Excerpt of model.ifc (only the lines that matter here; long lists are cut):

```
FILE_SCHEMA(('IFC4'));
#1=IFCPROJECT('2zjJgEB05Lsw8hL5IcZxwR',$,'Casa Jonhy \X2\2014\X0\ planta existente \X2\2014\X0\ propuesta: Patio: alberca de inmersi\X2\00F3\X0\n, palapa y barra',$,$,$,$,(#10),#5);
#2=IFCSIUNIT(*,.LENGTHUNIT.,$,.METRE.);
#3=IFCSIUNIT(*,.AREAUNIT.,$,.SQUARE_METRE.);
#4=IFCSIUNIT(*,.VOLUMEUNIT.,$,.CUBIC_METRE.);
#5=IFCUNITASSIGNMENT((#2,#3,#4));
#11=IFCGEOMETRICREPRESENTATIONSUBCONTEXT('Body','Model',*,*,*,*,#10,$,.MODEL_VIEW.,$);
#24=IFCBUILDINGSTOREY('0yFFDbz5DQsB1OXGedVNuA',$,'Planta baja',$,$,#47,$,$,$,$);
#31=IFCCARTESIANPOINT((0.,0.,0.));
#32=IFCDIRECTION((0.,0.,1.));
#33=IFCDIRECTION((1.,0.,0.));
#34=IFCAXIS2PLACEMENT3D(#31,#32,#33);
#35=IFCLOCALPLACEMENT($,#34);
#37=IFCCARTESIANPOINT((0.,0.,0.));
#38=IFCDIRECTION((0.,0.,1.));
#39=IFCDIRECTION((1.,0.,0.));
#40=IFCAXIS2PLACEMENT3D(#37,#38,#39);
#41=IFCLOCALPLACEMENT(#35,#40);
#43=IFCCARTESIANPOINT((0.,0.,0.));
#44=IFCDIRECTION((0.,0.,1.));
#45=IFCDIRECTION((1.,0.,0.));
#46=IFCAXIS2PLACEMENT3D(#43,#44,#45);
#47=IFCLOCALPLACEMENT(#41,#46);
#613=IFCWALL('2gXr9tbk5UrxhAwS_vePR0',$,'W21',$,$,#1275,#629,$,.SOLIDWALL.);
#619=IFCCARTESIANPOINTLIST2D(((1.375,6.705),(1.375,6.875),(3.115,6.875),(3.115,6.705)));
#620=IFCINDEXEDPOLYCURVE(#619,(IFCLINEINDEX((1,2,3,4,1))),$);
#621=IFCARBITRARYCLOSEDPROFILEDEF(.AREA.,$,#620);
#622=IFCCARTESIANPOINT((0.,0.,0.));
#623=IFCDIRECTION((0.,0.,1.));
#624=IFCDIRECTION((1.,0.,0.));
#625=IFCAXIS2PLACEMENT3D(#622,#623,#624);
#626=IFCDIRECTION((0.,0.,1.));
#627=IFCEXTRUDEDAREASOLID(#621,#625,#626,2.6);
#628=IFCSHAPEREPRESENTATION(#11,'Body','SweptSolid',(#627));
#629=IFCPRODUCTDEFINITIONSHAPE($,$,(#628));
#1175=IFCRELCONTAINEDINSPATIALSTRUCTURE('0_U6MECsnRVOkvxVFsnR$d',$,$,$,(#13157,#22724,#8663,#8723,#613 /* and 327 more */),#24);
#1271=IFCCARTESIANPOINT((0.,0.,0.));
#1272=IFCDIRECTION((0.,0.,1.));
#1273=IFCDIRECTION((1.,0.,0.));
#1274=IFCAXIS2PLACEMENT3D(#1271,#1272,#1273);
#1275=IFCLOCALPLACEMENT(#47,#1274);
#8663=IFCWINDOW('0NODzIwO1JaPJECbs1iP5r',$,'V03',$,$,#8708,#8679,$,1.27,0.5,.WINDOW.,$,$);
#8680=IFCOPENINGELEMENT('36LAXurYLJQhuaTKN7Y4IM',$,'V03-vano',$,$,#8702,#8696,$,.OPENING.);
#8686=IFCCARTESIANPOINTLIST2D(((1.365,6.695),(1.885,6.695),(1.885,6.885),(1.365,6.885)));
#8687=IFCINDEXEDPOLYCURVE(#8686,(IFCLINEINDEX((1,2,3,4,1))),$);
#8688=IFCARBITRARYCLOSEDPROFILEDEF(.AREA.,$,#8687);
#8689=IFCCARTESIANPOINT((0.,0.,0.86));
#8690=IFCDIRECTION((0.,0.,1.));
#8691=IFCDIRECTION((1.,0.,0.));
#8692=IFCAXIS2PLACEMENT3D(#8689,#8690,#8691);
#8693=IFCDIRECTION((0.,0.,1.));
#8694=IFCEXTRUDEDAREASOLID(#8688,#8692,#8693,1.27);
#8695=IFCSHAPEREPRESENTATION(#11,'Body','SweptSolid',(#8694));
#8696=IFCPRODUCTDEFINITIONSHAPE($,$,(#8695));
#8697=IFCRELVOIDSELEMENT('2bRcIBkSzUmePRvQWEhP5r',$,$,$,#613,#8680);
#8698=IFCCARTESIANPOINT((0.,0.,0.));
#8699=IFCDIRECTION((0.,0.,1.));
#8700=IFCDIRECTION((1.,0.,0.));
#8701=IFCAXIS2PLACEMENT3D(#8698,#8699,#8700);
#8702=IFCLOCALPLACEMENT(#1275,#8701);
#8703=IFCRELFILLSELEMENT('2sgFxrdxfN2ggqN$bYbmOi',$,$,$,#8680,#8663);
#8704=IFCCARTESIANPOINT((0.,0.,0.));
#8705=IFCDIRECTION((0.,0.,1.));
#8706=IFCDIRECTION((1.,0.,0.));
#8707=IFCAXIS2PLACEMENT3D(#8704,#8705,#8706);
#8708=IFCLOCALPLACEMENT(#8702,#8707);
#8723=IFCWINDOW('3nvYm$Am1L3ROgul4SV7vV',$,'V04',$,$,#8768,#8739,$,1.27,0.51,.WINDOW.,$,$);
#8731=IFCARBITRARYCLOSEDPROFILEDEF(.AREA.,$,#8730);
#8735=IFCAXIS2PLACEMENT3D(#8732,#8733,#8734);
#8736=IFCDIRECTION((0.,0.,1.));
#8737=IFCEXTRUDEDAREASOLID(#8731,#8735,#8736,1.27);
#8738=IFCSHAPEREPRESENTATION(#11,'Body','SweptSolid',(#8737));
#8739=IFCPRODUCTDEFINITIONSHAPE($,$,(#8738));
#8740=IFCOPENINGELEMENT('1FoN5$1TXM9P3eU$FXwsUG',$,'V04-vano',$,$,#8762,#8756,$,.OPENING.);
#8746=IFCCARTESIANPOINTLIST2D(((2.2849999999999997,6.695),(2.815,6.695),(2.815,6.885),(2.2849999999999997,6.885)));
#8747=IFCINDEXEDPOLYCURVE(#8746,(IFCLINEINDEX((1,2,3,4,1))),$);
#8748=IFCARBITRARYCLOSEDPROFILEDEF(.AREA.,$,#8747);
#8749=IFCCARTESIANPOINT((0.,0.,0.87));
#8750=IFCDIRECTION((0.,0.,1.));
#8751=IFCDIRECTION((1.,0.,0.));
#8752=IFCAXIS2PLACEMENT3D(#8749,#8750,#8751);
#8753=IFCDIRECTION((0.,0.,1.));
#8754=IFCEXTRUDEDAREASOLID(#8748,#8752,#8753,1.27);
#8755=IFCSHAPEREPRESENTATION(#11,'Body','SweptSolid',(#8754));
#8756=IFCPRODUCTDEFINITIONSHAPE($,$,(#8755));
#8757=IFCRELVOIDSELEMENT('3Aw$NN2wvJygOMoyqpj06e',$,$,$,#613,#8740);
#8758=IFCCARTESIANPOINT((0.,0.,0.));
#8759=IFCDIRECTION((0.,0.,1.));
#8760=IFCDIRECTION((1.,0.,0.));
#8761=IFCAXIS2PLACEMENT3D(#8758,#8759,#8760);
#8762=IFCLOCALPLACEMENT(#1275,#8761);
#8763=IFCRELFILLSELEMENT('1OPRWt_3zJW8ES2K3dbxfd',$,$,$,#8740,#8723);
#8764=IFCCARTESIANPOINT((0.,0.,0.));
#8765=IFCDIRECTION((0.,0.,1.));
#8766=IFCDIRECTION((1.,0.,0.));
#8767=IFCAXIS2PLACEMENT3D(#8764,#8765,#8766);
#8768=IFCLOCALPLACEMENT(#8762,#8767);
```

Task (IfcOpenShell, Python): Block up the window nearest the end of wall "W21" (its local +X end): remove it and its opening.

```python
import ifcopenshell
import ifcopenshell.api.feature
import ifcopenshell.api.root
import ifcopenshell.geom
import ifcopenshell.util.shape

model = ifcopenshell.open("model.ifc")
settings = ifcopenshell.geom.settings()


def volume(element):
    """Net volume in cubic metres, openings subtracted."""
    shape = ifcopenshell.geom.create_shape(settings, element)
    return ifcopenshell.util.shape.get_volume(shape.geometry)


window = model.by_guid("3nvYm$Am1L3ROgul4SV7vV")
opening = window.FillsVoids[0].RelatingOpeningElement
wall = opening.VoidsElements[0].RelatingBuildingElement
before = volume(wall)

ifcopenshell.api.root.remove_product(model, product=window)
ifcopenshell.api.feature.remove_feature(model, feature=opening)

after = volume(wall)

print(f"wall volume {before:.3f} -> {after:.3f} m3")

model.write("model_edited.ifc")
```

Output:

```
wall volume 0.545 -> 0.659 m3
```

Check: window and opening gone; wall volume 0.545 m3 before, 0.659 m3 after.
